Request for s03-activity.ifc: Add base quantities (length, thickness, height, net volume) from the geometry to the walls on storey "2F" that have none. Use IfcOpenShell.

First a look at what the model holds.

```python
import ifcopenshell
import ifcopenshell.util.element
import ifcopenshell.util.unit

model = ifcopenshell.open("s03-activity.ifc")
print(model.schema)
for unit_type in ("LENGTHUNIT", "AREAUNIT", "VOLUMEUNIT"):
    print(unit_type, ifcopenshell.util.unit.calculate_unit_scale(model, unit_type))
storey = next(s for s in model.by_type("IfcBuildingStorey") if s.Name == "2F")
walls = [e for e in ifcopenshell.util.element.get_decomposition(storey) if e.is_a("IfcWall")]
for e in sorted(walls, key=lambda e: e.id()):
    print(e.id(), e.is_a(), e.Name, list(ifcopenshell.util.element.get_psets(e, qtos_only=True)), sep=" | ")
```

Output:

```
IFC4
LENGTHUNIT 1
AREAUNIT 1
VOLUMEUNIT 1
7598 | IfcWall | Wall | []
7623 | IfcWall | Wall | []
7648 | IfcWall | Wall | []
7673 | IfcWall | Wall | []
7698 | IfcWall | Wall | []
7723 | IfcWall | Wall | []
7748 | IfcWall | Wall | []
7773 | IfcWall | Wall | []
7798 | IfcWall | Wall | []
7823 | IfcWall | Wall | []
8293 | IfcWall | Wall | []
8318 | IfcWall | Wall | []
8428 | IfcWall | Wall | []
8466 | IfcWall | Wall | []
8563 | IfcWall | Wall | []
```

```python
import ifcopenshell
import ifcopenshell.api.pset
import ifcopenshell.geom
import ifcopenshell.util.element
import ifcopenshell.util.shape
import ifcopenshell.util.unit

model = ifcopenshell.open("s03-activity.ifc")
unit_scale = ifcopenshell.util.unit.calculate_unit_scale(model)
volume_scale = ifcopenshell.util.unit.calculate_unit_scale(model, "VOLUMEUNIT")
settings = ifcopenshell.geom.settings()

storey = next(s for s in model.by_type("IfcBuildingStorey") if s.Name == "2F")
walls = [e for e in ifcopenshell.util.element.get_decomposition(storey) if e.is_a("IfcWall")]

for e in sorted(walls, key=lambda e: e.id()):
    if ifcopenshell.util.element.get_psets(e, qtos_only=True, should_inherit=False):
        continue
    # Geometry comes back in metres, in the element's own axes.
    shape = ifcopenshell.geom.create_shape(settings, e)
    values = {
        "Length": ifcopenshell.util.shape.get_x(shape.geometry) / unit_scale,
        "Width": ifcopenshell.util.shape.get_y(shape.geometry) / unit_scale,
        "Height": ifcopenshell.util.shape.get_z(shape.geometry) / unit_scale,
        "NetVolume": ifcopenshell.util.shape.get_volume(shape.geometry) / volume_scale,
    }
    qto = ifcopenshell.api.pset.add_qto(model, product=e, name="Qto_WallBaseQuantities")
    ifcopenshell.api.pset.edit_qto(model, qto=qto, properties=values)
    print(e.id(), {k: round(v, 3) for k, v in values.items()})

model.write("s03-activity_edited.ifc")
```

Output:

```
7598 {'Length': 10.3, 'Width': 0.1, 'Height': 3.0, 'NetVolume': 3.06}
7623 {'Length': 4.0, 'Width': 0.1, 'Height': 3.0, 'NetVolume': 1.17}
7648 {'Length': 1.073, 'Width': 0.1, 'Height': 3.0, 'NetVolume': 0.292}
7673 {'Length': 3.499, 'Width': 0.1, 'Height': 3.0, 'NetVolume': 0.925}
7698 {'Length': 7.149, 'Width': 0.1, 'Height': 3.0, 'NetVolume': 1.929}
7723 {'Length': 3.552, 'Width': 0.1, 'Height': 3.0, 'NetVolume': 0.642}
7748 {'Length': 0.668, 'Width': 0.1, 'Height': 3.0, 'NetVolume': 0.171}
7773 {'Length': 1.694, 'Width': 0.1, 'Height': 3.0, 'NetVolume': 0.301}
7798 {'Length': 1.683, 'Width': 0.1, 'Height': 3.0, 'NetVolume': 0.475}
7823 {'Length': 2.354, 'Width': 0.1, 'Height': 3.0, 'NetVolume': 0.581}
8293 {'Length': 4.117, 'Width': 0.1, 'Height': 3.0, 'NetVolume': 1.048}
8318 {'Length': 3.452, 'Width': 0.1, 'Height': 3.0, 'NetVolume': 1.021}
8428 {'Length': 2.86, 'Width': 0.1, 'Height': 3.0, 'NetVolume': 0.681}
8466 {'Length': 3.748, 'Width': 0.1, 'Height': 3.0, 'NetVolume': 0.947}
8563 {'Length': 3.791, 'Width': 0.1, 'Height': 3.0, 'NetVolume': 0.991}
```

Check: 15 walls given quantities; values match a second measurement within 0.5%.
